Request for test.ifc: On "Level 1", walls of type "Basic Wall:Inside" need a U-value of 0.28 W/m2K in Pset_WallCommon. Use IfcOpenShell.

First a look at what the model holds.

```python
import ifcopenshell
import ifcopenshell.util.element

model = ifcopenshell.open("test.ifc")
print(model.schema)
storey = next(s for s in model.by_type("IfcBuildingStorey") if s.Name == "Level 1")
walls = [e for e in ifcopenshell.util.element.get_decomposition(storey) if e.is_a("IfcWall")]
seen = {}
for e in walls:
    element_type = ifcopenshell.util.element.get_type(e)
    key = (element_type.Name if element_type != e and element_type else None, ifcopenshell.util.element.get_pset(e, "Pset_WallCommon", "ThermalTransmittance"))
    seen[key] = seen.get(key, 0) + 1
for (name, value), count in sorted(seen.items(), key=str):
    print(count, "x", name, "|", value)
```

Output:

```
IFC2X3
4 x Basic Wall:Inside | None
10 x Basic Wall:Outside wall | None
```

```python
import ifcopenshell
import ifcopenshell.api.pset
import ifcopenshell.util.element

model = ifcopenshell.open("test.ifc")

storey = next(s for s in model.by_type("IfcBuildingStorey") if s.Name == "Level 1")
walls = [e for e in ifcopenshell.util.element.get_decomposition(storey) if e.is_a("IfcWall")]

count = 0
for e in walls:
    element_type = ifcopenshell.util.element.get_type(e)
    if element_type in (None, e) or element_type.Name != "Basic Wall:Inside":
        continue
    # add_pset returns the element's existing set when there is one.
    pset = ifcopenshell.api.pset.add_pset(model, product=e, name="Pset_WallCommon")
    ifcopenshell.api.pset.edit_pset(model, pset=pset, properties={"ThermalTransmittance": 0.28})
    count += 1

print(count, "walls updated")

model.write("test-out.ifc")
```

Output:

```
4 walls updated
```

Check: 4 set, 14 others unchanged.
